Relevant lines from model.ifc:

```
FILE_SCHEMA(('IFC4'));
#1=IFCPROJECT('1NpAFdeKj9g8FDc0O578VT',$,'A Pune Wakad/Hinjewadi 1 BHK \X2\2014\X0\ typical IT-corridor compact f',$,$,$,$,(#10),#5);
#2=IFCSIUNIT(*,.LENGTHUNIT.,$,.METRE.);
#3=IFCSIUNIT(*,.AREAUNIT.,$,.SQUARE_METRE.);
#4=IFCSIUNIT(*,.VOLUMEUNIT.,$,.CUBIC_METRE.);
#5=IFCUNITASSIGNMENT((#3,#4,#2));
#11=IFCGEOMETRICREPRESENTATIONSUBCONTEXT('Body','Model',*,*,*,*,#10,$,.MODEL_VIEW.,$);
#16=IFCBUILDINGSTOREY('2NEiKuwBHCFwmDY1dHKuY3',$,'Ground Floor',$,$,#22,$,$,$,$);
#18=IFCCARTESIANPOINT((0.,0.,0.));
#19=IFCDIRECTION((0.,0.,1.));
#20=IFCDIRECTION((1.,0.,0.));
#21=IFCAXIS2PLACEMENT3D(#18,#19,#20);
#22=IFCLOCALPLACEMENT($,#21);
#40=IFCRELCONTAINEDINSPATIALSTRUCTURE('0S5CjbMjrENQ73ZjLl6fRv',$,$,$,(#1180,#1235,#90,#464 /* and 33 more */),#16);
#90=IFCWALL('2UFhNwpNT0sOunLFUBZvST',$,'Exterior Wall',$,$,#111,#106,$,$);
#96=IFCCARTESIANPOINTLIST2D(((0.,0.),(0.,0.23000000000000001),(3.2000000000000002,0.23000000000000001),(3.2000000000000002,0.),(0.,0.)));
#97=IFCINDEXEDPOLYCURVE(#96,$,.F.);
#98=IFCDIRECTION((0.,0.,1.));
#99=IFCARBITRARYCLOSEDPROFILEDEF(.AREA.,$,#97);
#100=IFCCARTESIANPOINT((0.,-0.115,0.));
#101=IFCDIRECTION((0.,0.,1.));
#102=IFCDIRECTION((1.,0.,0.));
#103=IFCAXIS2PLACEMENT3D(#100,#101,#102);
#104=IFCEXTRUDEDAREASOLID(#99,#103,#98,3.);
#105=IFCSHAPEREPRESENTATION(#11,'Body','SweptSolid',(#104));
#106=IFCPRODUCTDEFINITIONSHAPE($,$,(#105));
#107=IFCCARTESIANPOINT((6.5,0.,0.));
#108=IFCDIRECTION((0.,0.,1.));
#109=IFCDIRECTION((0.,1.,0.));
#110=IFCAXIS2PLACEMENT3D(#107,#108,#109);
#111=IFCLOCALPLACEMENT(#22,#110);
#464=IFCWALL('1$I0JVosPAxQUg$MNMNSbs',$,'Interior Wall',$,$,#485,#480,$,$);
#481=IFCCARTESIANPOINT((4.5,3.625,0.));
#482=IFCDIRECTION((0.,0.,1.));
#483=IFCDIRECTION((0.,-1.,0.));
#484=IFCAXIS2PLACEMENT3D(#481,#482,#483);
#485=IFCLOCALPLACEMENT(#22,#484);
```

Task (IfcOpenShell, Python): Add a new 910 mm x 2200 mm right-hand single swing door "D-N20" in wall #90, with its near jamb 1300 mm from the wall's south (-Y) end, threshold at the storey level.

```python
import numpy as np
import ifcopenshell
import ifcopenshell.api.feature
import ifcopenshell.api.geometry
import ifcopenshell.api.root
import ifcopenshell.api.spatial
import ifcopenshell.geom
import ifcopenshell.util.element
import ifcopenshell.util.placement
import ifcopenshell.util.representation
import ifcopenshell.util.shape
import ifcopenshell.util.unit

model = ifcopenshell.open("model.ifc")
unit_scale = ifcopenshell.util.unit.calculate_unit_scale(model)
settings = ifcopenshell.geom.settings()


def volume(element):
    """Net volume in cubic metres, openings subtracted."""
    shape = ifcopenshell.geom.create_shape(settings, element)
    return ifcopenshell.util.shape.get_volume(shape.geometry)


wall = model.by_guid("2UFhNwpNT0sOunLFUBZvST")
storey = ifcopenshell.util.element.get_container(wall, ifc_class="IfcBuildingStorey")
context = ifcopenshell.util.representation.get_context(model, "Model", "Body", "MODEL_VIEW")
before = volume(wall)

width, height, from_end, sill = 0.91, 2.2, 1.3, 0.0  # metres

# The wall runs along its own X axis, and the end named is its -X end.
wall_shape = ifcopenshell.geom.create_shape(settings, wall)
x, y, z = ifcopenshell.util.shape.get_vertices(wall_shape.geometry).T
start = x.min() + from_end
face, thickness = float(y.min()), float(y.max() - y.min())
wall_matrix = ifcopenshell.util.placement.get_local_placement(wall.ObjectPlacement)
level = ifcopenshell.util.placement.get_local_placement(storey.ObjectPlacement)[2, 3]


def in_wall(x, y):
    """Placement at x, y metres in the wall's axes, at sill height."""
    matrix = wall_matrix.copy()
    matrix[:, 3] = wall_matrix @ np.array([x / unit_scale, y / unit_scale, 0.0, 1.0])
    matrix[2, 3] = level + sill / unit_scale
    return matrix


# Opening: a box that overshoots both wall faces by 50 mm.
opening = ifcopenshell.api.root.create_entity(model, ifc_class="IfcOpeningElement", predefined_type="OPENING")
box = ifcopenshell.api.geometry.add_wall_representation(
    model, context=context, length=width, height=height, thickness=thickness + 0.1
)
ifcopenshell.api.geometry.assign_representation(model, product=opening, representation=box)
ifcopenshell.api.geometry.edit_object_placement(model, product=opening, matrix=in_wall(start, face - 0.05), is_si=False)
ifcopenshell.api.feature.add_feature(model, feature=opening, element=wall)

door = ifcopenshell.api.root.create_entity(model, ifc_class="IfcDoor", name="D-N20", predefined_type="DOOR")
door.OverallWidth, door.OverallHeight = width / unit_scale, height / unit_scale
door.OperationType = "SINGLE_SWING_RIGHT"
body = ifcopenshell.api.geometry.add_door_representation(
    model,
    context=context,
    overall_width=door.OverallWidth,
    overall_height=door.OverallHeight,
    operation_type="SINGLE_SWING_RIGHT",
    lining_properties={"LiningDepth": thickness / unit_scale, "ThresholdDepth": thickness / unit_scale},
)
ifcopenshell.api.geometry.assign_representation(model, product=door, representation=body)
ifcopenshell.api.spatial.assign_container(model, products=[door], relating_structure=storey)
ifcopenshell.api.feature.add_filling(model, opening=opening, element=door)

# The lining spans the wall, so the door starts at the wall face.
ifcopenshell.api.geometry.edit_object_placement(model, product=door, matrix=in_wall(start, face), is_si=False)

after = volume(wall)

print(f"wall volume {before:.3f} -> {after:.3f} m3")

model.write("model-out.ifc")
```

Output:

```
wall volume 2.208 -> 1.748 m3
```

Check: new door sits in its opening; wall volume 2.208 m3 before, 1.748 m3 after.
